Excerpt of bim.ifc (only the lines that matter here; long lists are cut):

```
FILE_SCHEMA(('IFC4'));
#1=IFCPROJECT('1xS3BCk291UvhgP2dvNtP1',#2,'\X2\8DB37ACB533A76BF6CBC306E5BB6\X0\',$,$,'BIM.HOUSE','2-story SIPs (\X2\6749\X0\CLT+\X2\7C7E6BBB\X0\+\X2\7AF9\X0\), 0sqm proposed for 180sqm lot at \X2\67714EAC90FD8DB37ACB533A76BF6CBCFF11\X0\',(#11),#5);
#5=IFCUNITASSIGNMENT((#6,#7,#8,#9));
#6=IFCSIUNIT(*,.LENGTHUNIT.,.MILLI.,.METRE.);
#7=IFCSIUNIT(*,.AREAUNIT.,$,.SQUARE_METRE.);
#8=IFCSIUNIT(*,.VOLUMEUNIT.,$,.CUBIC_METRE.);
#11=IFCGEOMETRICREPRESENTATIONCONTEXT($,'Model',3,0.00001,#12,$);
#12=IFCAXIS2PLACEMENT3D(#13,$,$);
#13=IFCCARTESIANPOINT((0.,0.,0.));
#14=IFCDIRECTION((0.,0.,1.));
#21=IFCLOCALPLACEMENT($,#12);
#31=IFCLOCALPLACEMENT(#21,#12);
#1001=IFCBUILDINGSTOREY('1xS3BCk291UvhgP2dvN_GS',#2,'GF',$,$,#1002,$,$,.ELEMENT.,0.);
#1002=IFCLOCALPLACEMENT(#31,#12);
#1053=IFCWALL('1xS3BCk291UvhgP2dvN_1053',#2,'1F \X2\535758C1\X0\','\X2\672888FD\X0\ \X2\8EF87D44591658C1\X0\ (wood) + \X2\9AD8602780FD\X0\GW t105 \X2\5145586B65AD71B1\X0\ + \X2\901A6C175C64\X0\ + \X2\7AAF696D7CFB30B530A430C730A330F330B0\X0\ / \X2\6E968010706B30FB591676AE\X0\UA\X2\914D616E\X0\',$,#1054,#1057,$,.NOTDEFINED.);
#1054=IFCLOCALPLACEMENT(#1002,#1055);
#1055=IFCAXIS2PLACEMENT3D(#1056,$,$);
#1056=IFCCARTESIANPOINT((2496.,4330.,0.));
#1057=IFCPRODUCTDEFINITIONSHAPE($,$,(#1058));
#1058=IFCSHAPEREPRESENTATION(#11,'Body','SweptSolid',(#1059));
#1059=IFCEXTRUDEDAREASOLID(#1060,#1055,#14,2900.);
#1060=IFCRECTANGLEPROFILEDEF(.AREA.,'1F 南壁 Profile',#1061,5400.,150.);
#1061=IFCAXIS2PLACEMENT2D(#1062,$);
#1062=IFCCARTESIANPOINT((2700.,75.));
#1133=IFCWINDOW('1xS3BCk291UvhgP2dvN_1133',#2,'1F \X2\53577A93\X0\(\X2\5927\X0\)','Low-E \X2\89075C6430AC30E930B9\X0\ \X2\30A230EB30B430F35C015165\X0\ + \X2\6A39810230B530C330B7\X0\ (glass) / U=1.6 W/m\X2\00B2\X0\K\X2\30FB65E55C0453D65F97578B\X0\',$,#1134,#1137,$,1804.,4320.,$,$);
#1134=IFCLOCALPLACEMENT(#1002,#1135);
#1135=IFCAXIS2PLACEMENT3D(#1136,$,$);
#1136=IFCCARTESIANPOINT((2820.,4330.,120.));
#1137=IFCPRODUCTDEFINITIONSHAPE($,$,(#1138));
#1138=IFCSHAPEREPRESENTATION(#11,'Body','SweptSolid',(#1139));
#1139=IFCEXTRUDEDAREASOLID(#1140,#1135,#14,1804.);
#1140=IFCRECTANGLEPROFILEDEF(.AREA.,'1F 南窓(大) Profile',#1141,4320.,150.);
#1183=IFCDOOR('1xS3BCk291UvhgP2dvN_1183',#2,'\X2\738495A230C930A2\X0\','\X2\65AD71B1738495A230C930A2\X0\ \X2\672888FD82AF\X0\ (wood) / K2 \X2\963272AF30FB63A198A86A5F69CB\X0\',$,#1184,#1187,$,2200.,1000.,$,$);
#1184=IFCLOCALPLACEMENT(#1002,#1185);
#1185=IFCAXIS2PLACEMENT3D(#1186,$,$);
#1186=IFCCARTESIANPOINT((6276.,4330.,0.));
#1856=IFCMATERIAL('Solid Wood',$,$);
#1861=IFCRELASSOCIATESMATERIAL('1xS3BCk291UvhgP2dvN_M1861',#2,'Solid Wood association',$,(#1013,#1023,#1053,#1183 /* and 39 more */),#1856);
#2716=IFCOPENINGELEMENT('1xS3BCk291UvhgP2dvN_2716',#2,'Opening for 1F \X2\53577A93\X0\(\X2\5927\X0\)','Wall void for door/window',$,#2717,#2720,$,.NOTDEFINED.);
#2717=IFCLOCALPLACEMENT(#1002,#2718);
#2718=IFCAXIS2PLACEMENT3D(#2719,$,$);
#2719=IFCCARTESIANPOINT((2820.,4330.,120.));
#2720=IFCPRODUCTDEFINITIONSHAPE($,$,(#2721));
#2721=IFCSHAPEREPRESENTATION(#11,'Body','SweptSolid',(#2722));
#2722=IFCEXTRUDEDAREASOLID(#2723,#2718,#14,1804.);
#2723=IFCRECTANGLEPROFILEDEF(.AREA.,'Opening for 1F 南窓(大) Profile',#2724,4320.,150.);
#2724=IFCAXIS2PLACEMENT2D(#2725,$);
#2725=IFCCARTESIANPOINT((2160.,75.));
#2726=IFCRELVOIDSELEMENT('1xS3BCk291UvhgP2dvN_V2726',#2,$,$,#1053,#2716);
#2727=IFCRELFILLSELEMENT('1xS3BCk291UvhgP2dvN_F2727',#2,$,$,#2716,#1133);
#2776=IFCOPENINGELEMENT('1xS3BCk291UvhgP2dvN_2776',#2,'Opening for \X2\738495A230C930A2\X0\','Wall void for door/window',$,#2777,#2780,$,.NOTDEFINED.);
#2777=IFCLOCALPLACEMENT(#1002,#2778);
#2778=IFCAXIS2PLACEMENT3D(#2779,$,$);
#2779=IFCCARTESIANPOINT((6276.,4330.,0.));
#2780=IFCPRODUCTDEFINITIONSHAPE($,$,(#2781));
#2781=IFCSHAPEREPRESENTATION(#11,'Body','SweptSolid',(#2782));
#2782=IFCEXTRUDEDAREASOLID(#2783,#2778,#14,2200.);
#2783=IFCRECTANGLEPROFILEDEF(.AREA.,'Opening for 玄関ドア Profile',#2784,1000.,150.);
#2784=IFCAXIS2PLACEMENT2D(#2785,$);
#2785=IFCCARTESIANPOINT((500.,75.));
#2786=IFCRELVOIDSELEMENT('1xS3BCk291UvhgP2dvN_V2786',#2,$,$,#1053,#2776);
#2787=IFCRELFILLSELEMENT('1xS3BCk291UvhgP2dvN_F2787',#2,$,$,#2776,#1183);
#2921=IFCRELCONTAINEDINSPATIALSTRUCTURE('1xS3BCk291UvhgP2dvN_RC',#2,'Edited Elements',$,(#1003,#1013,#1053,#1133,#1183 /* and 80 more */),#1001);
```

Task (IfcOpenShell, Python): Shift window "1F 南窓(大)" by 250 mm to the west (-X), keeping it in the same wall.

```python
import ifcopenshell
import ifcopenshell.api.geometry
import ifcopenshell.util.placement
import ifcopenshell.util.unit

model = ifcopenshell.open("bim.ifc")
unit_scale = ifcopenshell.util.unit.calculate_unit_scale(model)

window = model.by_id(1133)
opening = window.FillsVoids[0].RelatingOpeningElement
wall = opening.VoidsElements[0].RelatingBuildingElement

wall_matrix = ifcopenshell.util.placement.get_local_placement(wall.ObjectPlacement)
shift = wall_matrix[:3, 0] * -0.25 / unit_scale
before = ifcopenshell.util.placement.get_local_placement(window.ObjectPlacement)[:3, 3].copy()

# The window is not placed relative to its opening, so move both.
for product in (opening, window):
    matrix = ifcopenshell.util.placement.get_local_placement(product.ObjectPlacement)
    matrix[:3, 3] += shift
    ifcopenshell.api.geometry.edit_object_placement(model, product=product, matrix=matrix, is_si=False)

after = ifcopenshell.util.placement.get_local_placement(window.ObjectPlacement)[:3, 3]
print("window moved by", (after - before).round(3) + 0.0)

model.write("bim_v2.ifc")
```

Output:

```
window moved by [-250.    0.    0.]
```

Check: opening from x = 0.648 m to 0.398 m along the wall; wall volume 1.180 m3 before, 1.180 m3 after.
